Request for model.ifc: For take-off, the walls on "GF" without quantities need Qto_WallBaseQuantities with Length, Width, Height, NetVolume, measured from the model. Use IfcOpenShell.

First a look at what the model holds.

```python
import ifcopenshell
import ifcopenshell.util.element
import ifcopenshell.util.unit

model = ifcopenshell.open("model.ifc")
print(model.schema)
for unit_type in ("LENGTHUNIT", "AREAUNIT", "VOLUMEUNIT"):
    print(unit_type, ifcopenshell.util.unit.calculate_unit_scale(model, unit_type))
storey = next(s for s in model.by_type("IfcBuildingStorey") if s.Name == "GF")
walls = [e for e in ifcopenshell.util.element.get_decomposition(storey) if e.is_a("IfcWall")]
for e in sorted(walls, key=lambda e: e.id()):
    print(e.id(), e.is_a(), e.Name, list(ifcopenshell.util.element.get_psets(e, qtos_only=True)), sep=" | ")
```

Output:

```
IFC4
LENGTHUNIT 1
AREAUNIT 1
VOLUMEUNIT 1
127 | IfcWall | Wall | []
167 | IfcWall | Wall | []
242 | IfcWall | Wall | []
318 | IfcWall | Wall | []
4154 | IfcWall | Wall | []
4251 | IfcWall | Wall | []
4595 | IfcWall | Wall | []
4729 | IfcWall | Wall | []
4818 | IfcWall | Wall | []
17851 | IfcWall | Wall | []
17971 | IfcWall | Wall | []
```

```python
import ifcopenshell
import ifcopenshell.api.pset
import ifcopenshell.geom
import ifcopenshell.util.element
import ifcopenshell.util.shape
import ifcopenshell.util.unit

model = ifcopenshell.open("model.ifc")
unit_scale = ifcopenshell.util.unit.calculate_unit_scale(model)
volume_scale = ifcopenshell.util.unit.calculate_unit_scale(model, "VOLUMEUNIT")
settings = ifcopenshell.geom.settings()

storey = next(s for s in model.by_type("IfcBuildingStorey") if s.Name == "GF")
walls = [e for e in ifcopenshell.util.element.get_decomposition(storey) if e.is_a("IfcWall")]

for e in sorted(walls, key=lambda e: e.id()):
    if ifcopenshell.util.element.get_psets(e, qtos_only=True, should_inherit=False):
        continue
    # Geometry comes back in metres, in the element's own axes.
    shape = ifcopenshell.geom.create_shape(settings, e)
    values = {
        "Length": ifcopenshell.util.shape.get_x(shape.geometry) / unit_scale,
        "Width": ifcopenshell.util.shape.get_y(shape.geometry) / unit_scale,
        "Height": ifcopenshell.util.shape.get_z(shape.geometry) / unit_scale,
        "NetVolume": ifcopenshell.util.shape.get_volume(shape.geometry) / volume_scale,
    }
    qto = ifcopenshell.api.pset.add_qto(model, product=e, name="Qto_WallBaseQuantities")
    ifcopenshell.api.pset.edit_qto(model, qto=qto, properties=values)
    print(e.id(), {k: round(v, 3) for k, v in values.items()})

model.write("model_v2.ifc")
```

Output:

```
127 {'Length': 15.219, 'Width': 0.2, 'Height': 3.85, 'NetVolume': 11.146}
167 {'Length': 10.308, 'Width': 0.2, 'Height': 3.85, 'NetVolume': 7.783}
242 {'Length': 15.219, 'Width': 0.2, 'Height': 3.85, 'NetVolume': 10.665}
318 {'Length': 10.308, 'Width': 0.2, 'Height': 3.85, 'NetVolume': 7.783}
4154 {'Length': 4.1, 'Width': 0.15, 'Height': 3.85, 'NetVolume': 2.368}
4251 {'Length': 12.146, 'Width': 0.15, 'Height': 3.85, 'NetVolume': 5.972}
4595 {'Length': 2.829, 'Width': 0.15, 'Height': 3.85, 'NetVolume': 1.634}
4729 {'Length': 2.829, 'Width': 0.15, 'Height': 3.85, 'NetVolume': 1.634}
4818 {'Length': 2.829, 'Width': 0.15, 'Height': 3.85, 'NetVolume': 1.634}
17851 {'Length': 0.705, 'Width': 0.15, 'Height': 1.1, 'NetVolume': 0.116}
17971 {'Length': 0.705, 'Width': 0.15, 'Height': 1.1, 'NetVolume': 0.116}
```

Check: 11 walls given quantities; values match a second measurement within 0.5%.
